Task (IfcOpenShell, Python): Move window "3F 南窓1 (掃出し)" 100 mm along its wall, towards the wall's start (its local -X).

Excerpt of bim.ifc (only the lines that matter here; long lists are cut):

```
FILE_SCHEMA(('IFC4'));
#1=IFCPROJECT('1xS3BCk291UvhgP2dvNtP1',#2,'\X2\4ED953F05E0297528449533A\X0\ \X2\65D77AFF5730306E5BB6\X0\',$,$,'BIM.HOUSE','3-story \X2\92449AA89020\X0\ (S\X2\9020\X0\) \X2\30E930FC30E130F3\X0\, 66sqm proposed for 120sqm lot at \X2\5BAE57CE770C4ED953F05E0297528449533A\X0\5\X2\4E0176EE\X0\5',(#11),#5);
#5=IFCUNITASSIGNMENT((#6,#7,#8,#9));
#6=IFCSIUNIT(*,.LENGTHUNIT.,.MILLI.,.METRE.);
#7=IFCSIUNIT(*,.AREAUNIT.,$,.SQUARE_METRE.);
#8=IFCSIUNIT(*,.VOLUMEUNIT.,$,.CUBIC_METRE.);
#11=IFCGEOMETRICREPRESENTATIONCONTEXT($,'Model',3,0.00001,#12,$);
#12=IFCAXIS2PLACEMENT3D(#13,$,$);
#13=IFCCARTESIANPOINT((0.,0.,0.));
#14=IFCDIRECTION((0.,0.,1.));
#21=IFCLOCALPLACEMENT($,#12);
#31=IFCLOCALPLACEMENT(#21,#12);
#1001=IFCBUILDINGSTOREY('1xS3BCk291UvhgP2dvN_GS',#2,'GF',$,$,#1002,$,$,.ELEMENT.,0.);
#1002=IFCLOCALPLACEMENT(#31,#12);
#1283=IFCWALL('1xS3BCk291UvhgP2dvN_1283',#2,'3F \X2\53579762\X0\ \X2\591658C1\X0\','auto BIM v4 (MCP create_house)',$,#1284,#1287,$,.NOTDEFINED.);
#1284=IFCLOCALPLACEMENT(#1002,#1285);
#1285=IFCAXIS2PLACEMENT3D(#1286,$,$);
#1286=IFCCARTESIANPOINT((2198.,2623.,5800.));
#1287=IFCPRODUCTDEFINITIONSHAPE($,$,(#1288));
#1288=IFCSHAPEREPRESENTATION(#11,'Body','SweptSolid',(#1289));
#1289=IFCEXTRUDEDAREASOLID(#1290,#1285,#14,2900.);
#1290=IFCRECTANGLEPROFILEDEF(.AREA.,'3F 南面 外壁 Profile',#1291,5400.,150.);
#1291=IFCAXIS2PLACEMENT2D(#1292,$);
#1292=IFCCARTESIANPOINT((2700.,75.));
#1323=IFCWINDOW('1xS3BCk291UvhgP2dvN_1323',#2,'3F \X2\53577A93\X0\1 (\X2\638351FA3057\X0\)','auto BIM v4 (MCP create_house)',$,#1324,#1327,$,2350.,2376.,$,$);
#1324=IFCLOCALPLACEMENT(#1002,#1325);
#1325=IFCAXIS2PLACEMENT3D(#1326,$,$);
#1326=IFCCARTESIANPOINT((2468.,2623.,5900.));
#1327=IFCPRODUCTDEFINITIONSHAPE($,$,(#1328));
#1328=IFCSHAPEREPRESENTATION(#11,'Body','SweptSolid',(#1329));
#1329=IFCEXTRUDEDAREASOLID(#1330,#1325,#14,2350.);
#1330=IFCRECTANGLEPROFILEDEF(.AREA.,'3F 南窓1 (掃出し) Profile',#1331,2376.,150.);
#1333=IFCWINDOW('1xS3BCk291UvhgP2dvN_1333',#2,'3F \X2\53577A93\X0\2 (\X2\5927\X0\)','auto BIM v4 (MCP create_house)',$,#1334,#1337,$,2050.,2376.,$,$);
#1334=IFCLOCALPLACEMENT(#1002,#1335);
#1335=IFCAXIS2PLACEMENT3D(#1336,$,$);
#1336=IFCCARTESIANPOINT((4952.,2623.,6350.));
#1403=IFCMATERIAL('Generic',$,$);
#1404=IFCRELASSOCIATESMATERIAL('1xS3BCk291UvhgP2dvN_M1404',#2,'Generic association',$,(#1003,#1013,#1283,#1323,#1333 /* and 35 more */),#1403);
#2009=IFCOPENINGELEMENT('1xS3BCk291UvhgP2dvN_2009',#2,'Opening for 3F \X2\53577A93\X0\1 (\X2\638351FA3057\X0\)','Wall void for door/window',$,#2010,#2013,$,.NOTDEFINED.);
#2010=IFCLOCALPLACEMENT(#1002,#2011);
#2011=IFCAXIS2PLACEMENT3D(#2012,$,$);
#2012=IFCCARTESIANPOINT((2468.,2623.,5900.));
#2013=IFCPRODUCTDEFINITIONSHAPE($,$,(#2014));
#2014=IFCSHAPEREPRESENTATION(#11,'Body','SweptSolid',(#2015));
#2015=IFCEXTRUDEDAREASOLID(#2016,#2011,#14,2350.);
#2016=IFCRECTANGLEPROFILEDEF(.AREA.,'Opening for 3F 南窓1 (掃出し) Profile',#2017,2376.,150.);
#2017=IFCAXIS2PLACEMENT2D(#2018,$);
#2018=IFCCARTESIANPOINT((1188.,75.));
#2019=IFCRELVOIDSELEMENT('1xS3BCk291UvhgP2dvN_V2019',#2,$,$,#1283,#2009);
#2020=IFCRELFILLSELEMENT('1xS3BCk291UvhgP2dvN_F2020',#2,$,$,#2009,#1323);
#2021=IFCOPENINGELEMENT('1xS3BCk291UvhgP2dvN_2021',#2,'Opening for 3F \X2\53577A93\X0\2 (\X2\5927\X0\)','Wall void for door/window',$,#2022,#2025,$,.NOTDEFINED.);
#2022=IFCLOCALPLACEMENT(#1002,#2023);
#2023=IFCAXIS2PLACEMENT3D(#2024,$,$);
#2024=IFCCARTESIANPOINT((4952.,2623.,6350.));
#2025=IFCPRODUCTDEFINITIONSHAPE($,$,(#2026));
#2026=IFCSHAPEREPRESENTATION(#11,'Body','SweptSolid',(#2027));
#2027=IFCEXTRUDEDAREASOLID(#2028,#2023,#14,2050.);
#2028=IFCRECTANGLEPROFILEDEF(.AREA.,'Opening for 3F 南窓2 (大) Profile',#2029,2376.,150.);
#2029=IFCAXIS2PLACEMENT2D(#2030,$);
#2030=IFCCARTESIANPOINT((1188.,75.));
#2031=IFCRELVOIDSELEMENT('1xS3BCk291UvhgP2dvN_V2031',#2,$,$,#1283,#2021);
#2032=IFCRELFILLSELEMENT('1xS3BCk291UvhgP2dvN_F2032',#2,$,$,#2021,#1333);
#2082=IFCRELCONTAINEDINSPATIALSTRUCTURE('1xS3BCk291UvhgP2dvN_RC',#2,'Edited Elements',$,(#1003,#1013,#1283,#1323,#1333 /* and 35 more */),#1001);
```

```python
import ifcopenshell
import ifcopenshell.api.geometry
import ifcopenshell.util.placement
import ifcopenshell.util.unit

model = ifcopenshell.open("bim.ifc")
unit_scale = ifcopenshell.util.unit.calculate_unit_scale(model)

window = model.by_guid("1xS3BCk291UvhgP2dvN_1323")
opening = window.FillsVoids[0].RelatingOpeningElement
wall = opening.VoidsElements[0].RelatingBuildingElement

wall_matrix = ifcopenshell.util.placement.get_local_placement(wall.ObjectPlacement)
shift = wall_matrix[:3, 0] * -0.1 / unit_scale
before = ifcopenshell.util.placement.get_local_placement(window.ObjectPlacement)[:3, 3].copy()

# The window is not placed relative to its opening, so move both.
for product in (opening, window):
    matrix = ifcopenshell.util.placement.get_local_placement(product.ObjectPlacement)
    matrix[:3, 3] += shift
    ifcopenshell.api.geometry.edit_object_placement(model, product=product, matrix=matrix, is_si=False)

after = ifcopenshell.util.placement.get_local_placement(window.ObjectPlacement)[:3, 3]
print("window moved by", (after - before).round(3) + 0.0)

model.write("bim_edited.ifc")
```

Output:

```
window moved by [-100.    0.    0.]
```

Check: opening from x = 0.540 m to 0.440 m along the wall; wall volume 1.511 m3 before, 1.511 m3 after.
